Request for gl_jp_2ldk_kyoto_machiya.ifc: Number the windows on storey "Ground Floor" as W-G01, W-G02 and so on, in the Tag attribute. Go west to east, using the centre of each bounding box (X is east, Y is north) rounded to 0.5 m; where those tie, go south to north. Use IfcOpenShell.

First a look at what the model holds.

```python
import ifcopenshell
import ifcopenshell.util.element
import ifcopenshell.util.placement

model = ifcopenshell.open("gl_jp_2ldk_kyoto_machiya.ifc")
print(model.schema)
storey = next(s for s in model.by_type("IfcBuildingStorey") if s.Name == "Ground Floor")
windows = [e for e in ifcopenshell.util.element.get_decomposition(storey) if e.is_a("IfcWindow")]
for e in sorted(windows, key=lambda e: e.id()):
    origin = ifcopenshell.util.placement.get_local_placement(e.ObjectPlacement)[:3, 3]
    print(e.id(), e.Tag, e.Name, origin.round(2) + 0.0, sep=" | ")
```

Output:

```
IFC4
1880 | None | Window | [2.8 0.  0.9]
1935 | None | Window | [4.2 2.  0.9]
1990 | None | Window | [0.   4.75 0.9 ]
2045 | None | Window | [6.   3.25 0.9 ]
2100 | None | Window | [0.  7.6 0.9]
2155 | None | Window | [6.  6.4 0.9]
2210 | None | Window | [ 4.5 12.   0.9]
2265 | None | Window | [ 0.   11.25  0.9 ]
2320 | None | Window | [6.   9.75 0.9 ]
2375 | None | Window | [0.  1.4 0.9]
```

```python
import ifcopenshell
import ifcopenshell.geom
import ifcopenshell.util.element
import ifcopenshell.util.shape

model = ifcopenshell.open("gl_jp_2ldk_kyoto_machiya.ifc")
settings = ifcopenshell.geom.settings()
settings.set("use-world-coords", True)


def centre(element):
    shape = ifcopenshell.geom.create_shape(settings, element)
    return ifcopenshell.util.shape.get_bbox_centroid(shape.geometry)


storey = next(s for s in model.by_type("IfcBuildingStorey") if s.Name == "Ground Floor")
windows = [e for e in ifcopenshell.util.element.get_decomposition(storey) if e.is_a("IfcWindow")]

# Insertion points can sit at a corner or the storey origin, so sort by the geometry (in metres).
centres = {e: centre(e) for e in windows}
windows.sort(key=lambda e: (round(centres[e][0] / 0.5), centres[e][1]))

for i, e in enumerate(windows, start=1):
    number = f"W-G{i:02d}"
    e.Tag = number
    print(e.id(), number)

model.write("gl_jp_2ldk_kyoto_machiya_edited.ifc")
```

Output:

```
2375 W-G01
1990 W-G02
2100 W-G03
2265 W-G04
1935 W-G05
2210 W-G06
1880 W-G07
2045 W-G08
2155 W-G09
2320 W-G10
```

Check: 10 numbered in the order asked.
